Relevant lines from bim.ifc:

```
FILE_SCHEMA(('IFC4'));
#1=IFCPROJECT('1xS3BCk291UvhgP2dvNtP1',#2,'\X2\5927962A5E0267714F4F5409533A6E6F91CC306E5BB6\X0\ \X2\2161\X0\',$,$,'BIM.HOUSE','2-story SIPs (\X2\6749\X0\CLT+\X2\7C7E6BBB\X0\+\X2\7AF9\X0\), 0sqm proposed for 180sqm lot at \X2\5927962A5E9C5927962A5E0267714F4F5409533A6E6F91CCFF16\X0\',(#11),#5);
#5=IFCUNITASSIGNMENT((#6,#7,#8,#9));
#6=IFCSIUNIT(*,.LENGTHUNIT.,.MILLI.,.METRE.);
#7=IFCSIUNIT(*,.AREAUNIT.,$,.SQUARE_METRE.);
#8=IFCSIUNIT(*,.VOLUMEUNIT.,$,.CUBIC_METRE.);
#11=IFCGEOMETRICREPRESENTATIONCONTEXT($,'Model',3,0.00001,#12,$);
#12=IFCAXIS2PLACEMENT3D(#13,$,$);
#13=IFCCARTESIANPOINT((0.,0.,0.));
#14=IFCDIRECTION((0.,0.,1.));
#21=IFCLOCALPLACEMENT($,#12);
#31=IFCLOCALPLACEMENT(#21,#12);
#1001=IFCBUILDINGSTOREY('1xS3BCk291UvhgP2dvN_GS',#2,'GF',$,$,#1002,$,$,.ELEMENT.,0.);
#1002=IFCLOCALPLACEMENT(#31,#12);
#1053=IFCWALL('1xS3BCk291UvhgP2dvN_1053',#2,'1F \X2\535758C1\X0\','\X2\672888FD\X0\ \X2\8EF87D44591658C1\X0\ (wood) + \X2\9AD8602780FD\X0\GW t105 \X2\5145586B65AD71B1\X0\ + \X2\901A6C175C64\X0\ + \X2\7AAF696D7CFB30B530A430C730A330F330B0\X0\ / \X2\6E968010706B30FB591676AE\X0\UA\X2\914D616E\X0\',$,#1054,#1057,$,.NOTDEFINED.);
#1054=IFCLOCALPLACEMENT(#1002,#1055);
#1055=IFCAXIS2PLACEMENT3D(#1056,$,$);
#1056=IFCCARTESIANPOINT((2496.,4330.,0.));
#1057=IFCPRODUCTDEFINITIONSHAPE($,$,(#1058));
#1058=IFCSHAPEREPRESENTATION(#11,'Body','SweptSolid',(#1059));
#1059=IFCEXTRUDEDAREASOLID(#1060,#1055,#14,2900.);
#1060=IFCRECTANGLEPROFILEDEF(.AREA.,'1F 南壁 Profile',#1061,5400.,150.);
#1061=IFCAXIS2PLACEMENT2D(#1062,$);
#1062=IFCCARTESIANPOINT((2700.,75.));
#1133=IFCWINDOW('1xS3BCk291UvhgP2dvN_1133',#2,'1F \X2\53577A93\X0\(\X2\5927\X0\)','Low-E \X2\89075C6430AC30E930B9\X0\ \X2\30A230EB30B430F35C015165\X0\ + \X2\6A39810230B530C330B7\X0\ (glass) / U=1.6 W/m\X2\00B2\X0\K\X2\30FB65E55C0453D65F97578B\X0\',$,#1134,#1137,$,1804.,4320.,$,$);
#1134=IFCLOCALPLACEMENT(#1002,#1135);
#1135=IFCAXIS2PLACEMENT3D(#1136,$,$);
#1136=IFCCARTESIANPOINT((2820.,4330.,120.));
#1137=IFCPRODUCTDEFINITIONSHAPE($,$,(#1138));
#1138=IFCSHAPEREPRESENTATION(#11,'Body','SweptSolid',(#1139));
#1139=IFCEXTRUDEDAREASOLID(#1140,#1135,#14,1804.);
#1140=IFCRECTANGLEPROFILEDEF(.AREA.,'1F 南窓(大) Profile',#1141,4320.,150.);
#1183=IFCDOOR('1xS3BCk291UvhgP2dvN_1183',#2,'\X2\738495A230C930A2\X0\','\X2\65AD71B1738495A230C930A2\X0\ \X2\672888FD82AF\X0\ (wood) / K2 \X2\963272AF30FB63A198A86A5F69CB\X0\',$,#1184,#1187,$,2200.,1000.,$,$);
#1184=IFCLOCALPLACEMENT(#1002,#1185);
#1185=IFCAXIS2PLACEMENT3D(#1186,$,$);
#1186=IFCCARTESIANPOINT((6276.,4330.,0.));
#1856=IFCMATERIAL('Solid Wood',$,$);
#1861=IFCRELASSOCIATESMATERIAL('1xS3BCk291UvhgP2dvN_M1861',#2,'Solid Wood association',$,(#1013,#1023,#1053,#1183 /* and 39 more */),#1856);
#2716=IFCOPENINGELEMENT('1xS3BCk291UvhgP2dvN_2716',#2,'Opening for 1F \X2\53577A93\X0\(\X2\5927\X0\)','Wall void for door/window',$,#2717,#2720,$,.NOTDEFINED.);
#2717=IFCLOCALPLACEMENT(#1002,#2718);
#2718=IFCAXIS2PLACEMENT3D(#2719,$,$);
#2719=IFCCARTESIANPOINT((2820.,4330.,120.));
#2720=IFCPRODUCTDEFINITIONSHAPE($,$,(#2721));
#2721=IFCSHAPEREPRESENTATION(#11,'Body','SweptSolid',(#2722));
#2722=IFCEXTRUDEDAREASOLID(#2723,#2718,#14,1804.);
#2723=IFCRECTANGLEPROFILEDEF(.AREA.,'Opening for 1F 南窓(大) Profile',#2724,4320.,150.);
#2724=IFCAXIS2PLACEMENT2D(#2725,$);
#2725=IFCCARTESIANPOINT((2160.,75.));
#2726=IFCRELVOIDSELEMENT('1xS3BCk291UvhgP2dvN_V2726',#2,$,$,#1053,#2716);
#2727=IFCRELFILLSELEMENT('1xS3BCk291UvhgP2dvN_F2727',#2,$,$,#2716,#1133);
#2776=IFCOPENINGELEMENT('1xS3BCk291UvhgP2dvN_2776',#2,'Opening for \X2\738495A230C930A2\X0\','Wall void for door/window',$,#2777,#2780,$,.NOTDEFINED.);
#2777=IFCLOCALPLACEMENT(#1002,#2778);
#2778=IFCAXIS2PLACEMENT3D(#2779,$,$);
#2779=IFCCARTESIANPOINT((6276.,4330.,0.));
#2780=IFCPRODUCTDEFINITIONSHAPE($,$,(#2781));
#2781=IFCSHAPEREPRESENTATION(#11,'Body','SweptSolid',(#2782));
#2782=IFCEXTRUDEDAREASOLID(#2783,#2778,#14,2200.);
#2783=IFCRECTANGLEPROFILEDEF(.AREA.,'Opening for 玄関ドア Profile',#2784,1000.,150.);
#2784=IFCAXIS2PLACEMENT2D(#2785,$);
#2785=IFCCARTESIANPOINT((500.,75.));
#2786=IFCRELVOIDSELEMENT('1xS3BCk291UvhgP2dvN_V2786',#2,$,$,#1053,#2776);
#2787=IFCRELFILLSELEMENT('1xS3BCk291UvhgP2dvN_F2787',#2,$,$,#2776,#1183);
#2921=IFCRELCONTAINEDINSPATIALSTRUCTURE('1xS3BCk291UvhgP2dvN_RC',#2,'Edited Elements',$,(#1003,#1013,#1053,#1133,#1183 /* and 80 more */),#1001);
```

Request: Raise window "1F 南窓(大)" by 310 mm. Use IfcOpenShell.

```python
import numpy as np
import ifcopenshell
import ifcopenshell.api.geometry
import ifcopenshell.util.placement
import ifcopenshell.util.unit

model = ifcopenshell.open("bim.ifc")
unit_scale = ifcopenshell.util.unit.calculate_unit_scale(model)

window = model.by_guid("1xS3BCk291UvhgP2dvN_1133")
opening = window.FillsVoids[0].RelatingOpeningElement
dz = 310.0

shift = np.array([0.0, 0.0, dz])
# The window is not placed relative to its opening, so move both.
for product in (opening, window):
    matrix = ifcopenshell.util.placement.get_local_placement(product.ObjectPlacement)
    matrix[:3, 3] += shift
    ifcopenshell.api.geometry.edit_object_placement(model, product=product, matrix=matrix, is_si=False)

print(f"moved by {dz * unit_scale:+.3f} m")

model.write("bim_updated.ifc")
```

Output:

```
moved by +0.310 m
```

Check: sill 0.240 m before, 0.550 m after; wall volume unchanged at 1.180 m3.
